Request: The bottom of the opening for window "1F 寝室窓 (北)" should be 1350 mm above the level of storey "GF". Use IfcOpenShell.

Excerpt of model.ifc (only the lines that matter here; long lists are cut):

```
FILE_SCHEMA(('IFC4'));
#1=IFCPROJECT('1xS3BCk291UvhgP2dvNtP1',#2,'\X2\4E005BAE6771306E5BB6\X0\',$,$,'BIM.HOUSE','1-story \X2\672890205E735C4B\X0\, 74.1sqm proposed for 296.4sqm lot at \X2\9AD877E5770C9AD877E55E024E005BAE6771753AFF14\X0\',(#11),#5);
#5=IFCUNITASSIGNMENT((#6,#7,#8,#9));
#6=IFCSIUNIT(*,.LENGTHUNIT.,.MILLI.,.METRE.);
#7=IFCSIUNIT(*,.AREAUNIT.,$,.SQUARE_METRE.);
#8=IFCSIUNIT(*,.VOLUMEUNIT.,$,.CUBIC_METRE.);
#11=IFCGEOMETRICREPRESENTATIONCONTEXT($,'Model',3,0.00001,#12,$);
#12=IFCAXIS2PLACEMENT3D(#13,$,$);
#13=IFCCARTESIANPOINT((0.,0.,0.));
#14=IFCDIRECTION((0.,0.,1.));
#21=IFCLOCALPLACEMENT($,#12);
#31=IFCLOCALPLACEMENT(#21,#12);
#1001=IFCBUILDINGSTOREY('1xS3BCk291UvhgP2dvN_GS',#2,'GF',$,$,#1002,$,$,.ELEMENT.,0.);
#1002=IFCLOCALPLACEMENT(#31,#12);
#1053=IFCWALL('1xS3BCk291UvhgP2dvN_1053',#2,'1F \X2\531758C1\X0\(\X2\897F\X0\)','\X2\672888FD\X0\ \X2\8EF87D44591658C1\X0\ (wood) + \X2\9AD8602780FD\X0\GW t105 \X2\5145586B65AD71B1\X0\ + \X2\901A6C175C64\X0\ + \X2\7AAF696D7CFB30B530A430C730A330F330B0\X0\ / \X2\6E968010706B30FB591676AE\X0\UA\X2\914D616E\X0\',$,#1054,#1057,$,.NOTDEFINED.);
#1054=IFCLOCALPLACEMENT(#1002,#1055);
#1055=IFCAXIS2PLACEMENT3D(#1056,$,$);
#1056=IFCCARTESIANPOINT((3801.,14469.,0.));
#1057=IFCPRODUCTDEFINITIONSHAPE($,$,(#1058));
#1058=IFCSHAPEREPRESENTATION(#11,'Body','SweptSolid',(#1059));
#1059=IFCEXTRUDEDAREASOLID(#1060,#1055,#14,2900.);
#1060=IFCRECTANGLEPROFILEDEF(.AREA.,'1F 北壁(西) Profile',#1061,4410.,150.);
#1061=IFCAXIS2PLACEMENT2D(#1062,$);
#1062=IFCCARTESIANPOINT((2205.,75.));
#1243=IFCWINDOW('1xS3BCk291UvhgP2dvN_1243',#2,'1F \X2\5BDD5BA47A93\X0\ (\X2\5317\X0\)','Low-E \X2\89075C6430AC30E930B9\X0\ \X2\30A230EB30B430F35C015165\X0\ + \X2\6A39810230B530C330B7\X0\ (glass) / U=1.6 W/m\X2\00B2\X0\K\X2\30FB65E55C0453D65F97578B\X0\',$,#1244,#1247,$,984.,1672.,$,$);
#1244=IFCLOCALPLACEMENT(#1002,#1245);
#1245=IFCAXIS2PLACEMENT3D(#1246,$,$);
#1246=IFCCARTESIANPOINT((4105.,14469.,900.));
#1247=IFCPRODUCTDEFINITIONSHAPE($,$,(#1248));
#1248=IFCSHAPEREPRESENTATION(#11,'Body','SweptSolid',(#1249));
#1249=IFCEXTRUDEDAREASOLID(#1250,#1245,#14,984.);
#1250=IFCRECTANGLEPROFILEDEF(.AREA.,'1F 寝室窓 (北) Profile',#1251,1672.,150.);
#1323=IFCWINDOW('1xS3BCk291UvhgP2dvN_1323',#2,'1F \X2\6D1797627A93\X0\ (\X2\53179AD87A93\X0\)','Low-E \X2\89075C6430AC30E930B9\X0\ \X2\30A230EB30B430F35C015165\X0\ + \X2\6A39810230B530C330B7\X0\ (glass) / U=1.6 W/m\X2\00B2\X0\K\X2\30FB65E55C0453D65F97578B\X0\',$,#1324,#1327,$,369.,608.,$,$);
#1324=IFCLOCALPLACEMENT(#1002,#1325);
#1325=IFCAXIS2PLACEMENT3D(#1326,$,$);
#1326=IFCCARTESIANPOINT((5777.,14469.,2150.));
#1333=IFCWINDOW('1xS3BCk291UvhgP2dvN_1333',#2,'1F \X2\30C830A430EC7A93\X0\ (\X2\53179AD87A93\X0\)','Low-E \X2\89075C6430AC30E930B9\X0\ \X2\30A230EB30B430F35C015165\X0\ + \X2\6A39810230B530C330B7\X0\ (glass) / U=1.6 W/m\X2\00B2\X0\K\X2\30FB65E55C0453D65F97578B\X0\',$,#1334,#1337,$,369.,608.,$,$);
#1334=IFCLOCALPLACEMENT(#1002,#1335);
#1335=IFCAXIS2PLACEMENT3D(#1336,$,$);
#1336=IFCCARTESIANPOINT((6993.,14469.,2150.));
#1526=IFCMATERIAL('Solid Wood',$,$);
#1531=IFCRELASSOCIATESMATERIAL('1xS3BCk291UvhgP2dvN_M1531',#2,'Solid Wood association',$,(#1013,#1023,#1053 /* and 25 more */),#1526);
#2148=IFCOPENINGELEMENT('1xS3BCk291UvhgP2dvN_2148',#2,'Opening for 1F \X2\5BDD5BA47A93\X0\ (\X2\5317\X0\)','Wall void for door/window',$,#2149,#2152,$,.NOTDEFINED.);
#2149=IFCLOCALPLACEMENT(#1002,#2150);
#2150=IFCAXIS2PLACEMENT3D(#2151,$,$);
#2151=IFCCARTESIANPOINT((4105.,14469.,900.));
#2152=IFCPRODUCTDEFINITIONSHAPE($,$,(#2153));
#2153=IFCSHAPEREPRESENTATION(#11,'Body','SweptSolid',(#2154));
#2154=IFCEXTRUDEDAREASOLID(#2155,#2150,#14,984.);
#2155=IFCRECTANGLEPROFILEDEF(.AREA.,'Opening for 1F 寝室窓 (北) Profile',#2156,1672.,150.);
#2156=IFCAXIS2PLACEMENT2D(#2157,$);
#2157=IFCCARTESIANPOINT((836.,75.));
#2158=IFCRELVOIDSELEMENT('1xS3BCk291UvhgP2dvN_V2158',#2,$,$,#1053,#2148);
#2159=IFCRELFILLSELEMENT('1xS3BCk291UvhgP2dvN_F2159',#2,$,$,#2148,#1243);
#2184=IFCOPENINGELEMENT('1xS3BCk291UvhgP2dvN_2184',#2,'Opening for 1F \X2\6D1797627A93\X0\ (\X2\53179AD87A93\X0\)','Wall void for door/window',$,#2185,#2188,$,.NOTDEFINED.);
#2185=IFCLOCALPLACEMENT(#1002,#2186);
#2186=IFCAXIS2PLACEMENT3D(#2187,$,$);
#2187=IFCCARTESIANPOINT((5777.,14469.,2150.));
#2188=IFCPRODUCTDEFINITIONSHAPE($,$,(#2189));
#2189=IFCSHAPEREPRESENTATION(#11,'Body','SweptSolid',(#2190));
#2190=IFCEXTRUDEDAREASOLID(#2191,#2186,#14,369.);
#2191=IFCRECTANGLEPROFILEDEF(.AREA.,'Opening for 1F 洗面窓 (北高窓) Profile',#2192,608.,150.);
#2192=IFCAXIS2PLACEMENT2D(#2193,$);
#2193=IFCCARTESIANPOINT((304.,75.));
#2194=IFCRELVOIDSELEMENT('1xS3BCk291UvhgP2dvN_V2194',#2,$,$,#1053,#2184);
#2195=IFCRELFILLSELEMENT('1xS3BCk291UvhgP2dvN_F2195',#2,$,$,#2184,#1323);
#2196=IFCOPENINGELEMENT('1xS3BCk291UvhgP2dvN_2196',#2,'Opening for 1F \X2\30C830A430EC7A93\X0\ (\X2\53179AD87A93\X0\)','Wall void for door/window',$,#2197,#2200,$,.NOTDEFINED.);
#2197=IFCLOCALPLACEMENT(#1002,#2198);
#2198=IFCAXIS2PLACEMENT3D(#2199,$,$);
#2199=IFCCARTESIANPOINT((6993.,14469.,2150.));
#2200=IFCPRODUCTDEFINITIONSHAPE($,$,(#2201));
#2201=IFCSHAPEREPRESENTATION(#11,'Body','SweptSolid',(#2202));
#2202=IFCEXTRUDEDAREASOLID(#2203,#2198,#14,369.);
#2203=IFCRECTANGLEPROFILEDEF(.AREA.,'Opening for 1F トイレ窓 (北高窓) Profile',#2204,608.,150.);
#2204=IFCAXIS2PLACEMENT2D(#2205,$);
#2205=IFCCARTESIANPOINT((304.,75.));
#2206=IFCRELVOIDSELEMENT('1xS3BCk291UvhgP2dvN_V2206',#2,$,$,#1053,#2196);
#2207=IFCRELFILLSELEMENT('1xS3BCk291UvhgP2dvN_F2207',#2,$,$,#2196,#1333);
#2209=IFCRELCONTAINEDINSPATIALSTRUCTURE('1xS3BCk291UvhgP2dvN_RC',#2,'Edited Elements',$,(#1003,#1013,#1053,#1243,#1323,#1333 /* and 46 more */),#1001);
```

```python
import numpy as np
import ifcopenshell
import ifcopenshell.api.geometry
import ifcopenshell.geom
import ifcopenshell.util.element
import ifcopenshell.util.placement
import ifcopenshell.util.shape
import ifcopenshell.util.unit

model = ifcopenshell.open("model.ifc")
unit_scale = ifcopenshell.util.unit.calculate_unit_scale(model)

window = model.by_guid("1xS3BCk291UvhgP2dvN_1243")
opening = window.FillsVoids[0].RelatingOpeningElement
storey = ifcopenshell.util.element.get_container(window, ifc_class="IfcBuildingStorey")
level = ifcopenshell.util.placement.get_local_placement(storey.ObjectPlacement)[2, 3]

# The opening's origin need not be at the sill, so measure its lowest point.
shape = ifcopenshell.geom.create_shape(ifcopenshell.geom.settings(), opening)
bottom = ifcopenshell.util.shape.get_shape_bottom_elevation(shape, shape.geometry) / unit_scale
dz = level + 1.35 / unit_scale - bottom

shift = np.array([0.0, 0.0, dz])
# The window is not placed relative to its opening, so move both.
for product in (opening, window):
    matrix = ifcopenshell.util.placement.get_local_placement(product.ObjectPlacement)
    matrix[:3, 3] += shift
    ifcopenshell.api.geometry.edit_object_placement(model, product=product, matrix=matrix, is_si=False)

print(f"moved by {dz * unit_scale:+.3f} m")

model.write("model_v2.ifc")
```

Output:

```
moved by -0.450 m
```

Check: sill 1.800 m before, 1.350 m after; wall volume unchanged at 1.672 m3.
